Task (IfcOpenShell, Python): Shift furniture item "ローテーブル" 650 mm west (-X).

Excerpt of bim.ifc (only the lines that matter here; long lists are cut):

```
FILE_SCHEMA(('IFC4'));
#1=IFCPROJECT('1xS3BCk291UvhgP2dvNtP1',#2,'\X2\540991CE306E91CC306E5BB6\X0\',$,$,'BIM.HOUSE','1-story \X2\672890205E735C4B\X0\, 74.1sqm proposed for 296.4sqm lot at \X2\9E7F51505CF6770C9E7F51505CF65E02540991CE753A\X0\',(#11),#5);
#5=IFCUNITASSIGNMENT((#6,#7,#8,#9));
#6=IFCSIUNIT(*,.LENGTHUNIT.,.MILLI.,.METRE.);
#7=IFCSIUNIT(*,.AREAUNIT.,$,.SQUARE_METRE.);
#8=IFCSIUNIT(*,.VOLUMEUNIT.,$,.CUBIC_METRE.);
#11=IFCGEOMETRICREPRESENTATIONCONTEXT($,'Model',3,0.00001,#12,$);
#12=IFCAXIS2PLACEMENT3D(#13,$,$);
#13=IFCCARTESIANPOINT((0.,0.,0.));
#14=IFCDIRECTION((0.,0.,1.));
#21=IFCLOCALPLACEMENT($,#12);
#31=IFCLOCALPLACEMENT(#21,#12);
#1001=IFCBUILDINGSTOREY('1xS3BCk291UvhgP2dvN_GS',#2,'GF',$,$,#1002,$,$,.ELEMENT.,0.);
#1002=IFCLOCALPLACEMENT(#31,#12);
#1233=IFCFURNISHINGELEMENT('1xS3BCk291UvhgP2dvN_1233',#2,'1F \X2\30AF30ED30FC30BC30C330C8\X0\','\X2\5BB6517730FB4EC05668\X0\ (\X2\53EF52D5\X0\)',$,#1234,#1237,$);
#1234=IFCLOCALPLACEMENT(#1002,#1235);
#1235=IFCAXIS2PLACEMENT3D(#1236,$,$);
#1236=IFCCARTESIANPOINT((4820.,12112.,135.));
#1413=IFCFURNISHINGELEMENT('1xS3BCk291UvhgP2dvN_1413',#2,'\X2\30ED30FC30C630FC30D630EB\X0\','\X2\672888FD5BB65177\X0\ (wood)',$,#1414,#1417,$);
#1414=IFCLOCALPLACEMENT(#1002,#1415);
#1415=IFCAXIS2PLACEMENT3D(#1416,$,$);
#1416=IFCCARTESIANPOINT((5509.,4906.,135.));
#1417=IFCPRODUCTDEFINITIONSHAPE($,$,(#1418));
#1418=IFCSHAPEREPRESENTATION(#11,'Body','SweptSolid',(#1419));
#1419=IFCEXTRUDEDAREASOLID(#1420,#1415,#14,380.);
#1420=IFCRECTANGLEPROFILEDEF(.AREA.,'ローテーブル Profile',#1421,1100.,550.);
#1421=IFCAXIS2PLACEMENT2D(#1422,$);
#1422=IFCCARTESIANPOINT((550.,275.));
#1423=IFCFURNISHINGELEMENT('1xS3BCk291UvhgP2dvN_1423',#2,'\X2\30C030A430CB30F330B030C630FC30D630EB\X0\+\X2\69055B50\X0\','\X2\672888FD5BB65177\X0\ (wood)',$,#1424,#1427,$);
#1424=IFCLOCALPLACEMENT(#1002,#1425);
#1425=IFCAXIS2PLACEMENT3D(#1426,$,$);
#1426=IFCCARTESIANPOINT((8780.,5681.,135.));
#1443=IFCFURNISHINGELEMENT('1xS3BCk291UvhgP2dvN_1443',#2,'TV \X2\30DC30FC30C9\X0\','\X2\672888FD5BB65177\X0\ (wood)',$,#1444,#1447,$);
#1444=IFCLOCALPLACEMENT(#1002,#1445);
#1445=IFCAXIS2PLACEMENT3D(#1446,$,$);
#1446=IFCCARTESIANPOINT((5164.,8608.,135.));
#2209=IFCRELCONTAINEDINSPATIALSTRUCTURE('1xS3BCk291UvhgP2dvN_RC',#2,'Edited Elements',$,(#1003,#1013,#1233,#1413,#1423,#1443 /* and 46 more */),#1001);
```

```python
import ifcopenshell
import ifcopenshell.api.geometry
import ifcopenshell.util.placement

model = ifcopenshell.open("bim.ifc")

item = model.by_id(1413)
matrix = ifcopenshell.util.placement.get_local_placement(item.ObjectPlacement)
matrix[0, 3] -= 650.0
ifcopenshell.api.geometry.edit_object_placement(model, product=item, matrix=matrix, is_si=False)

print(ifcopenshell.util.placement.get_local_placement(item.ObjectPlacement).round(3) + 0.0)

model.write("bim_v2.ifc")
```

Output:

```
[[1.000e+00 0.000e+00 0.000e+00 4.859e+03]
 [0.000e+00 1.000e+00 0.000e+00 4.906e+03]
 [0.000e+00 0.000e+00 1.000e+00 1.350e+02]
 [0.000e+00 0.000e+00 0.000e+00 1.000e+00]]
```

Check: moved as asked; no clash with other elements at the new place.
